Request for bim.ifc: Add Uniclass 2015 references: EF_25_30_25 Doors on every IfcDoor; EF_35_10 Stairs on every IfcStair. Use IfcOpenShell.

First a look at what the model holds.

```python
import ifcopenshell

model = ifcopenshell.open("bim.ifc")
print(model.schema)
print("classifications:", [c.Name for c in model.by_type("IfcClassification")])
for ifc_class in ("IfcDoor", "IfcRoof", "IfcStair", "IfcWall", "IfcWindow"):
    print(ifc_class, len(model.by_type(ifc_class)))
```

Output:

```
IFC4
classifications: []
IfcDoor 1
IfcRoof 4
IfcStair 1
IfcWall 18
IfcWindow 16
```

```python
import ifcopenshell
import ifcopenshell.api.classification

model = ifcopenshell.open("bim.ifc")

system = ifcopenshell.api.classification.add_classification(model, classification="Uniclass 2015")

codes = {
    "IfcDoor": ("EF_25_30_25", "Doors"),
    "IfcStair": ("EF_35_10", "Stairs"),
}
for ifc_class, (code, name) in codes.items():
    products = model.by_type(ifc_class)
    ifcopenshell.api.classification.add_reference(
        model, products=products, classification=system, identification=code, name=name
    )
    print(code, len(products))

model.write("bim_rev.ifc")
```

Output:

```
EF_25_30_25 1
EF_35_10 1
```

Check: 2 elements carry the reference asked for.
